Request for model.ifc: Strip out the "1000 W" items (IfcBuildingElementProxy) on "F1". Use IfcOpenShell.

First a look at what the model holds.

```python
import ifcopenshell
import ifcopenshell.util.element

model = ifcopenshell.open("model.ifc")
print(model.schema)
storey = next(s for s in model.by_type("IfcBuildingStorey") if s.Name == "F1")
proxies = [e for e in ifcopenshell.util.element.get_decomposition(storey) if e.is_a("IfcBuildingElementProxy")]
seen = {}
for e in proxies:
    element_type = ifcopenshell.util.element.get_type(e)
    name = element_type.Name if element_type not in (None, e) else None
    seen[name] = seen.get(name, 0) + 1
for name, count in sorted(seen.items(), key=str):
    print(count, "x", name)
```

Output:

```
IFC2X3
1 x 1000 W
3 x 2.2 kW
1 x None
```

```python
import ifcopenshell
import ifcopenshell.api.root
import ifcopenshell.util.element

model = ifcopenshell.open("model.ifc")

storey = next(s for s in model.by_type("IfcBuildingStorey") if s.Name == "F1")
proxies = [e for e in ifcopenshell.util.element.get_decomposition(storey) if e.is_a("IfcBuildingElementProxy")]
targets = [e for e in proxies if (t := ifcopenshell.util.element.get_type(e)) not in (None, e) and t.Name == "1000 W"]

for e in targets:
    ifcopenshell.api.root.remove_product(model, product=e)
print(len(targets), "removed")

model.write("model_rev.ifc")
```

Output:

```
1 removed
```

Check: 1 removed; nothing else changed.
